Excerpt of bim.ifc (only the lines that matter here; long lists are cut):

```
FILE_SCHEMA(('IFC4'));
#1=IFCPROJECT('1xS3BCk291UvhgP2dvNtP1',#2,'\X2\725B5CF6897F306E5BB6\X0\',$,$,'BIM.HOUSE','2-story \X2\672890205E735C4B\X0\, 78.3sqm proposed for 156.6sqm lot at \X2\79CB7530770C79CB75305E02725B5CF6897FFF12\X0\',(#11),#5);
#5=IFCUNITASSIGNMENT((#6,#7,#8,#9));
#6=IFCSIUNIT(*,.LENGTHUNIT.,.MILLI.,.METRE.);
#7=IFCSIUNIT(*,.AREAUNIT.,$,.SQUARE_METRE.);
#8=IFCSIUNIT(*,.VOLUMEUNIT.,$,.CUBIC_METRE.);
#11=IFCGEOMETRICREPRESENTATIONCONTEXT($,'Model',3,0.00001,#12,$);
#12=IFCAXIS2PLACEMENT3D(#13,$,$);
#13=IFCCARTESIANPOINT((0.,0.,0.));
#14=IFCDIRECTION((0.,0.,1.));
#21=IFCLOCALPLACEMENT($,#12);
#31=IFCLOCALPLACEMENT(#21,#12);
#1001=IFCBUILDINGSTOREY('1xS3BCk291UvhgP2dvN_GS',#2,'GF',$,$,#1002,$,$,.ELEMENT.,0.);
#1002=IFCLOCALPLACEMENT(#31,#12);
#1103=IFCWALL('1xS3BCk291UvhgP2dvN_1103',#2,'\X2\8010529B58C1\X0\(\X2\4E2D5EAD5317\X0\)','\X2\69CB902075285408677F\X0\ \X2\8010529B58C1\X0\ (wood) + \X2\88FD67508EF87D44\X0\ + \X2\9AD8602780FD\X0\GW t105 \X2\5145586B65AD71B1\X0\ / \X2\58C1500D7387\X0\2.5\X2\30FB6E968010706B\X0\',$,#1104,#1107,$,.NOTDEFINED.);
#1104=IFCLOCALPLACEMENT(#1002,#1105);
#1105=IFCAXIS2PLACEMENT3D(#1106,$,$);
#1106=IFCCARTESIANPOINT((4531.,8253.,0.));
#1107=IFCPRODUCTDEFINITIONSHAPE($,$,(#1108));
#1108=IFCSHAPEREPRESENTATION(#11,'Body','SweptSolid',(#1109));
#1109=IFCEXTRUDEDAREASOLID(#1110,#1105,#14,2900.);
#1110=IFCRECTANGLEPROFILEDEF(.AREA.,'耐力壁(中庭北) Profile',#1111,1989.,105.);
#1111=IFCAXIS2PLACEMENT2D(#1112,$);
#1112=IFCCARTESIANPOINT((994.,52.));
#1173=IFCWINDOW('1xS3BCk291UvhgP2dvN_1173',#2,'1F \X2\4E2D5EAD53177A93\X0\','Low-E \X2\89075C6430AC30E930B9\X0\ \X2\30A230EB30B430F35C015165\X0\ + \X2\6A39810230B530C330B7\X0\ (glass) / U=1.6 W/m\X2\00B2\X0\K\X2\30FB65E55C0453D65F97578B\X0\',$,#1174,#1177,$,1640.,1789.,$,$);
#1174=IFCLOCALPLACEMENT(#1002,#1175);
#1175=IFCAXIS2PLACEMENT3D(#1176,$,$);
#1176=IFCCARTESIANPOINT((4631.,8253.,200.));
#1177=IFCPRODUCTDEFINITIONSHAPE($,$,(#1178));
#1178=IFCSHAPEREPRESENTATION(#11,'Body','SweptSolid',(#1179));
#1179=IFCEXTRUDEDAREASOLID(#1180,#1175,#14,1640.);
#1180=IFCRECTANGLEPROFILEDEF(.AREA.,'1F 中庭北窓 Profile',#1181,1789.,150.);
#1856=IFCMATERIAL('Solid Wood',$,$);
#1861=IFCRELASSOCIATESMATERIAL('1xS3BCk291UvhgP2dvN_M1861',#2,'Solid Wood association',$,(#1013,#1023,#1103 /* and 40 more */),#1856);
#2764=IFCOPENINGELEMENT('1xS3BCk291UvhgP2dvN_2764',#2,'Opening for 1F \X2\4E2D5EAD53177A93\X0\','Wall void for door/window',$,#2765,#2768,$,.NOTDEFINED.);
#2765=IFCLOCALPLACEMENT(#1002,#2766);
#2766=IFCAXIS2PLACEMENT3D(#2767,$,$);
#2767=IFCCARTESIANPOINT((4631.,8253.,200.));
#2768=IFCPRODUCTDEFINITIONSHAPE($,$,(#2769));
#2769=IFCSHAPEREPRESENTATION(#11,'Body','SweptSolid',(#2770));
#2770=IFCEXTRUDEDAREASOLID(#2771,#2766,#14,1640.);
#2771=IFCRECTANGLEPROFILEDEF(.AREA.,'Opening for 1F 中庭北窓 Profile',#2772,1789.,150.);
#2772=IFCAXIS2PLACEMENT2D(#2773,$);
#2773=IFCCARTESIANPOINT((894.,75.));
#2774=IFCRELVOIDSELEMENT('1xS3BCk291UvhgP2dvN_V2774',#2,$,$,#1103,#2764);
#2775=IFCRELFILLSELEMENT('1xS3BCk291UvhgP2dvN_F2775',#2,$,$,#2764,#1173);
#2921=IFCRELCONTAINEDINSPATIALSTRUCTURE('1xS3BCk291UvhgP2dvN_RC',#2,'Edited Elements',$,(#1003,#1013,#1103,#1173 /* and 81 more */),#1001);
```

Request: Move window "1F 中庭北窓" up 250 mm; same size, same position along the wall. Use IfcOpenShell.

```python
import numpy as np
import ifcopenshell
import ifcopenshell.api.geometry
import ifcopenshell.util.placement
import ifcopenshell.util.unit

model = ifcopenshell.open("bim.ifc")
unit_scale = ifcopenshell.util.unit.calculate_unit_scale(model)

window = model.by_guid("1xS3BCk291UvhgP2dvN_1173")
opening = window.FillsVoids[0].RelatingOpeningElement
dz = 250.0

shift = np.array([0.0, 0.0, dz])
# The window is not placed relative to its opening, so move both.
for product in (opening, window):
    matrix = ifcopenshell.util.placement.get_local_placement(product.ObjectPlacement)
    matrix[:3, 3] += shift
    ifcopenshell.api.geometry.edit_object_placement(model, product=product, matrix=matrix, is_si=False)

print(f"moved by {dz * unit_scale:+.3f} m")

model.write("bim-out.ifc")
```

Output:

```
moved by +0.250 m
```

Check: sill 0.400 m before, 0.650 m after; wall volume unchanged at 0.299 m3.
